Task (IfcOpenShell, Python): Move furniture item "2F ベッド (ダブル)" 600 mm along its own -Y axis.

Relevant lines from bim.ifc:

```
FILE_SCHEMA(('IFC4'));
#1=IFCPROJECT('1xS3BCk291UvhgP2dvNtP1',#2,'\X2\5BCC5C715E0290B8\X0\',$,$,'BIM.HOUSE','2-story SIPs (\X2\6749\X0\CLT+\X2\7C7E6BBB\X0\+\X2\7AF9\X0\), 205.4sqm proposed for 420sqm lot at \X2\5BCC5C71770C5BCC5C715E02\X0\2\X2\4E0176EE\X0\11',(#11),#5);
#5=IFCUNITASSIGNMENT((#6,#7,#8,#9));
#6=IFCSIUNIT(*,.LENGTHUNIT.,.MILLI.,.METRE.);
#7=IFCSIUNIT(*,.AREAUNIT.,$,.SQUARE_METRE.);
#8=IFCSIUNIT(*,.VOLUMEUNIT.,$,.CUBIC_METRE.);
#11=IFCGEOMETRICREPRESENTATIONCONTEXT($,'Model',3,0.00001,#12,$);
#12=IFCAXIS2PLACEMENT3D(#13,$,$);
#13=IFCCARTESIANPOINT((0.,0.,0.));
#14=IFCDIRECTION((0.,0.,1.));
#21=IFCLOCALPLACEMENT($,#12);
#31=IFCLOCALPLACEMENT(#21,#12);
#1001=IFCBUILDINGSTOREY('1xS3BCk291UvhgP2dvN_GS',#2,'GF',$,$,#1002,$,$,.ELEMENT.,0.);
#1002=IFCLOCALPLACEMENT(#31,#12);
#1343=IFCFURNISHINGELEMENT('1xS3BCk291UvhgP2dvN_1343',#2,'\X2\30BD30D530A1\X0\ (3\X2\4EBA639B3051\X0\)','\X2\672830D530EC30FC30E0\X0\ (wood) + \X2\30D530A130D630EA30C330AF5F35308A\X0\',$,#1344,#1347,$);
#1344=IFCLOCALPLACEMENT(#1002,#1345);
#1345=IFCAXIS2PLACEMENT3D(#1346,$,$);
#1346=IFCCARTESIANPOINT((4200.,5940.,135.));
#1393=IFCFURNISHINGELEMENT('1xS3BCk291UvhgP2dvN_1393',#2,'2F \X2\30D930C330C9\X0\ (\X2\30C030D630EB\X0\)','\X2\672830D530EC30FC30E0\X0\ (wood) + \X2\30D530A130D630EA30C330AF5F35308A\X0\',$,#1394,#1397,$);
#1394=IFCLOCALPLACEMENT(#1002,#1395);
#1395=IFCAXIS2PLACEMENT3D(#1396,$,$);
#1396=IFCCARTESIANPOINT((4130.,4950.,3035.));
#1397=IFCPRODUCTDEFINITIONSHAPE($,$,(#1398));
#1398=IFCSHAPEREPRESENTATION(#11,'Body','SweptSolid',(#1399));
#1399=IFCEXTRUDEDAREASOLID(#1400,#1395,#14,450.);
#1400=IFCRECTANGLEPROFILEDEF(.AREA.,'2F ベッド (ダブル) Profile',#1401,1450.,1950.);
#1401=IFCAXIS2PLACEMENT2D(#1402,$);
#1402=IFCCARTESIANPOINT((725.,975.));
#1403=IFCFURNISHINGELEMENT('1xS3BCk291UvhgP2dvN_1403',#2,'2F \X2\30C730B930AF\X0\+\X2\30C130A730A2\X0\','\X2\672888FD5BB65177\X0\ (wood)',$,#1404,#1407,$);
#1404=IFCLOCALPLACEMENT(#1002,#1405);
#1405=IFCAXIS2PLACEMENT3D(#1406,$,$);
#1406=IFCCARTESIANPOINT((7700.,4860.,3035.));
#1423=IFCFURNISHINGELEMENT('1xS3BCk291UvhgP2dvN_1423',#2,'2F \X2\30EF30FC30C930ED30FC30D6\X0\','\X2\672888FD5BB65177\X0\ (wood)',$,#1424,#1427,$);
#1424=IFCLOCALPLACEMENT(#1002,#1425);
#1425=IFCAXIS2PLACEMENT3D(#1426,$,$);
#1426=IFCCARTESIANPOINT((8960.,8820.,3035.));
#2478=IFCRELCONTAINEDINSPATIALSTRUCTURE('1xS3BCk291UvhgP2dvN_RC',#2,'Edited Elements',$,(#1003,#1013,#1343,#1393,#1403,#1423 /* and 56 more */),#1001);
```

```python
import ifcopenshell
import ifcopenshell.api.geometry
import ifcopenshell.util.placement
import ifcopenshell.util.unit

model = ifcopenshell.open("bim.ifc")
unit_scale = ifcopenshell.util.unit.calculate_unit_scale(model)

item = model.by_guid("1xS3BCk291UvhgP2dvN_1393")
matrix = ifcopenshell.util.placement.get_local_placement(item.ObjectPlacement)
matrix[:3, 3] -= matrix[:3, 1] * 0.6 / unit_scale
ifcopenshell.api.geometry.edit_object_placement(model, product=item, matrix=matrix, is_si=False)

print(ifcopenshell.util.placement.get_local_placement(item.ObjectPlacement).round(3) + 0.0)

model.write("bim_v2.ifc")
```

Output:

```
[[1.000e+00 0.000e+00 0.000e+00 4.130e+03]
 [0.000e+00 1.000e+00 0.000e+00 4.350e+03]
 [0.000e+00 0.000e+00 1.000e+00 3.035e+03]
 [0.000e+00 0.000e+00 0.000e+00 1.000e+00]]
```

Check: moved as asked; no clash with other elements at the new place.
